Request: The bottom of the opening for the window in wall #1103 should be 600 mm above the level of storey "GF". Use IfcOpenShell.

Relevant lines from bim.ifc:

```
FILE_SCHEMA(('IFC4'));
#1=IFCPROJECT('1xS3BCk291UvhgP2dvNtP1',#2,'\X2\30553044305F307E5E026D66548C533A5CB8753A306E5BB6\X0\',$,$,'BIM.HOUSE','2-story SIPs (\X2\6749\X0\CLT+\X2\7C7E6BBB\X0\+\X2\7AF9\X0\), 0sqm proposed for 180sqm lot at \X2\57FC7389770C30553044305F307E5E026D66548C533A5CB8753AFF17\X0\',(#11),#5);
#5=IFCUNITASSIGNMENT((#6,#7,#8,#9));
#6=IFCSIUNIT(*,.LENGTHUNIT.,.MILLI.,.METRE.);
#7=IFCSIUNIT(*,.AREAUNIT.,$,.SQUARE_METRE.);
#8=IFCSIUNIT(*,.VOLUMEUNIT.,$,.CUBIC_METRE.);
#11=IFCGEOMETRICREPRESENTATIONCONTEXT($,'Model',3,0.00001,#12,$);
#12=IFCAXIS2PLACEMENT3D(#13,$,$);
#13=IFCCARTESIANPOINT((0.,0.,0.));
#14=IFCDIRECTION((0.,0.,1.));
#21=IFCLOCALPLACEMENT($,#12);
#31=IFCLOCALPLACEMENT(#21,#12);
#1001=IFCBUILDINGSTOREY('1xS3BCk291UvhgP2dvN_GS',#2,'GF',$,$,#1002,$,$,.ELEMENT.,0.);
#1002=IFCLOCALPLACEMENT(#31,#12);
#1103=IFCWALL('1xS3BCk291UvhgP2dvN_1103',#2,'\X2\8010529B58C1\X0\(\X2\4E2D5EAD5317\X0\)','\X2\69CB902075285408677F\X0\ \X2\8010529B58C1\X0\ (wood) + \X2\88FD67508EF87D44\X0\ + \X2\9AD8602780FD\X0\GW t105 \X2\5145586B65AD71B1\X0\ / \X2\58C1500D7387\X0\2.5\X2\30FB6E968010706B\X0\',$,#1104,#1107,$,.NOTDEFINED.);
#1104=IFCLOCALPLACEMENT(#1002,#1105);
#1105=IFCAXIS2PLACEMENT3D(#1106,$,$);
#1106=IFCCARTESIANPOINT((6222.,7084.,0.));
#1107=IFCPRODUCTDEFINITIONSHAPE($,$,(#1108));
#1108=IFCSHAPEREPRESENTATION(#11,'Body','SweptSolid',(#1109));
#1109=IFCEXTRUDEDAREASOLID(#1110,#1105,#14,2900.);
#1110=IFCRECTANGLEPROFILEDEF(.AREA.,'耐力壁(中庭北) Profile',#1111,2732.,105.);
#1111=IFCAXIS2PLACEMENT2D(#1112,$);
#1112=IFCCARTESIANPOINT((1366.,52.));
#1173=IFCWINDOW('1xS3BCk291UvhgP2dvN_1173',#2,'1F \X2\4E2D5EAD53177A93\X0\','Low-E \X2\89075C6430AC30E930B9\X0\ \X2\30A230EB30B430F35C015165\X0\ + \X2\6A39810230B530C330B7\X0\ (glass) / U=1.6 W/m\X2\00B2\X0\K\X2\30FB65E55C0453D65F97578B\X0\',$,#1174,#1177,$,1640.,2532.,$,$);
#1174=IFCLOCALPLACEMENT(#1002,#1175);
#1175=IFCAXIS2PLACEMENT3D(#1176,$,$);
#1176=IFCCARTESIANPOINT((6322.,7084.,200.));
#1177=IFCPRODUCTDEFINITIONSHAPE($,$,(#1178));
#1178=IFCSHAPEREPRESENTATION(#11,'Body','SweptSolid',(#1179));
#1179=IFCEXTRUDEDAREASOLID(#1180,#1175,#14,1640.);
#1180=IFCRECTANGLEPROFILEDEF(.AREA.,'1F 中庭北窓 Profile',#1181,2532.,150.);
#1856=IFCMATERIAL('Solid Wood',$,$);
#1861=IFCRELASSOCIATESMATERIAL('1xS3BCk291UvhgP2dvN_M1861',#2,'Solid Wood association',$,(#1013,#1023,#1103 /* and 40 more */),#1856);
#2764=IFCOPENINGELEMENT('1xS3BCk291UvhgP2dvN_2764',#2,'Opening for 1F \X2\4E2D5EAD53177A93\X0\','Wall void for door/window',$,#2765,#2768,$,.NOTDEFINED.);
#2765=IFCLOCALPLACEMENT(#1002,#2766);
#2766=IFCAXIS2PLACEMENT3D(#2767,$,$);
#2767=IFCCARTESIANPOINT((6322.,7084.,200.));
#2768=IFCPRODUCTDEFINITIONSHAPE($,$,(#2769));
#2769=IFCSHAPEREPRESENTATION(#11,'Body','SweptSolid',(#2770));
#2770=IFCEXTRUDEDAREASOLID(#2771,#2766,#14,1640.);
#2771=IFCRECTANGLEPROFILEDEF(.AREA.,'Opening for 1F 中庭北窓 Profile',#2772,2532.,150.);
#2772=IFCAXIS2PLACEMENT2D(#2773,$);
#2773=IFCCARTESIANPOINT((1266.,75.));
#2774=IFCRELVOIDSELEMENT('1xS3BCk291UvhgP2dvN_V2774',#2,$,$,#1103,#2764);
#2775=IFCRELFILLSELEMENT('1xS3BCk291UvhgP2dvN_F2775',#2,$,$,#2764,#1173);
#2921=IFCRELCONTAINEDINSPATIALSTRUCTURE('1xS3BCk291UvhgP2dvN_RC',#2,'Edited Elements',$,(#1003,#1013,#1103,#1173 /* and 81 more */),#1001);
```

```python
import numpy as np
import ifcopenshell
import ifcopenshell.api.geometry
import ifcopenshell.geom
import ifcopenshell.util.element
import ifcopenshell.util.placement
import ifcopenshell.util.shape
import ifcopenshell.util.unit

model = ifcopenshell.open("bim.ifc")
unit_scale = ifcopenshell.util.unit.calculate_unit_scale(model)

window = model.by_guid("1xS3BCk291UvhgP2dvN_1173")
opening = window.FillsVoids[0].RelatingOpeningElement
storey = ifcopenshell.util.element.get_container(window, ifc_class="IfcBuildingStorey")
level = ifcopenshell.util.placement.get_local_placement(storey.ObjectPlacement)[2, 3]

# The opening's origin need not be at the sill, so measure its lowest point.
shape = ifcopenshell.geom.create_shape(ifcopenshell.geom.settings(), opening)
bottom = ifcopenshell.util.shape.get_shape_bottom_elevation(shape, shape.geometry) / unit_scale
dz = level + 600.0 - bottom

shift = np.array([0.0, 0.0, dz])
# The window is not placed relative to its opening, so move both.
for product in (opening, window):
    matrix = ifcopenshell.util.placement.get_local_placement(product.ObjectPlacement)
    matrix[:3, 3] += shift
    ifcopenshell.api.geometry.edit_object_placement(model, product=product, matrix=matrix, is_si=False)

print(f"moved by {dz * unit_scale:+.3f} m")

model.write("bim-out.ifc")
```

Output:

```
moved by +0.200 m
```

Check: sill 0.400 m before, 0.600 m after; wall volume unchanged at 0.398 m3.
